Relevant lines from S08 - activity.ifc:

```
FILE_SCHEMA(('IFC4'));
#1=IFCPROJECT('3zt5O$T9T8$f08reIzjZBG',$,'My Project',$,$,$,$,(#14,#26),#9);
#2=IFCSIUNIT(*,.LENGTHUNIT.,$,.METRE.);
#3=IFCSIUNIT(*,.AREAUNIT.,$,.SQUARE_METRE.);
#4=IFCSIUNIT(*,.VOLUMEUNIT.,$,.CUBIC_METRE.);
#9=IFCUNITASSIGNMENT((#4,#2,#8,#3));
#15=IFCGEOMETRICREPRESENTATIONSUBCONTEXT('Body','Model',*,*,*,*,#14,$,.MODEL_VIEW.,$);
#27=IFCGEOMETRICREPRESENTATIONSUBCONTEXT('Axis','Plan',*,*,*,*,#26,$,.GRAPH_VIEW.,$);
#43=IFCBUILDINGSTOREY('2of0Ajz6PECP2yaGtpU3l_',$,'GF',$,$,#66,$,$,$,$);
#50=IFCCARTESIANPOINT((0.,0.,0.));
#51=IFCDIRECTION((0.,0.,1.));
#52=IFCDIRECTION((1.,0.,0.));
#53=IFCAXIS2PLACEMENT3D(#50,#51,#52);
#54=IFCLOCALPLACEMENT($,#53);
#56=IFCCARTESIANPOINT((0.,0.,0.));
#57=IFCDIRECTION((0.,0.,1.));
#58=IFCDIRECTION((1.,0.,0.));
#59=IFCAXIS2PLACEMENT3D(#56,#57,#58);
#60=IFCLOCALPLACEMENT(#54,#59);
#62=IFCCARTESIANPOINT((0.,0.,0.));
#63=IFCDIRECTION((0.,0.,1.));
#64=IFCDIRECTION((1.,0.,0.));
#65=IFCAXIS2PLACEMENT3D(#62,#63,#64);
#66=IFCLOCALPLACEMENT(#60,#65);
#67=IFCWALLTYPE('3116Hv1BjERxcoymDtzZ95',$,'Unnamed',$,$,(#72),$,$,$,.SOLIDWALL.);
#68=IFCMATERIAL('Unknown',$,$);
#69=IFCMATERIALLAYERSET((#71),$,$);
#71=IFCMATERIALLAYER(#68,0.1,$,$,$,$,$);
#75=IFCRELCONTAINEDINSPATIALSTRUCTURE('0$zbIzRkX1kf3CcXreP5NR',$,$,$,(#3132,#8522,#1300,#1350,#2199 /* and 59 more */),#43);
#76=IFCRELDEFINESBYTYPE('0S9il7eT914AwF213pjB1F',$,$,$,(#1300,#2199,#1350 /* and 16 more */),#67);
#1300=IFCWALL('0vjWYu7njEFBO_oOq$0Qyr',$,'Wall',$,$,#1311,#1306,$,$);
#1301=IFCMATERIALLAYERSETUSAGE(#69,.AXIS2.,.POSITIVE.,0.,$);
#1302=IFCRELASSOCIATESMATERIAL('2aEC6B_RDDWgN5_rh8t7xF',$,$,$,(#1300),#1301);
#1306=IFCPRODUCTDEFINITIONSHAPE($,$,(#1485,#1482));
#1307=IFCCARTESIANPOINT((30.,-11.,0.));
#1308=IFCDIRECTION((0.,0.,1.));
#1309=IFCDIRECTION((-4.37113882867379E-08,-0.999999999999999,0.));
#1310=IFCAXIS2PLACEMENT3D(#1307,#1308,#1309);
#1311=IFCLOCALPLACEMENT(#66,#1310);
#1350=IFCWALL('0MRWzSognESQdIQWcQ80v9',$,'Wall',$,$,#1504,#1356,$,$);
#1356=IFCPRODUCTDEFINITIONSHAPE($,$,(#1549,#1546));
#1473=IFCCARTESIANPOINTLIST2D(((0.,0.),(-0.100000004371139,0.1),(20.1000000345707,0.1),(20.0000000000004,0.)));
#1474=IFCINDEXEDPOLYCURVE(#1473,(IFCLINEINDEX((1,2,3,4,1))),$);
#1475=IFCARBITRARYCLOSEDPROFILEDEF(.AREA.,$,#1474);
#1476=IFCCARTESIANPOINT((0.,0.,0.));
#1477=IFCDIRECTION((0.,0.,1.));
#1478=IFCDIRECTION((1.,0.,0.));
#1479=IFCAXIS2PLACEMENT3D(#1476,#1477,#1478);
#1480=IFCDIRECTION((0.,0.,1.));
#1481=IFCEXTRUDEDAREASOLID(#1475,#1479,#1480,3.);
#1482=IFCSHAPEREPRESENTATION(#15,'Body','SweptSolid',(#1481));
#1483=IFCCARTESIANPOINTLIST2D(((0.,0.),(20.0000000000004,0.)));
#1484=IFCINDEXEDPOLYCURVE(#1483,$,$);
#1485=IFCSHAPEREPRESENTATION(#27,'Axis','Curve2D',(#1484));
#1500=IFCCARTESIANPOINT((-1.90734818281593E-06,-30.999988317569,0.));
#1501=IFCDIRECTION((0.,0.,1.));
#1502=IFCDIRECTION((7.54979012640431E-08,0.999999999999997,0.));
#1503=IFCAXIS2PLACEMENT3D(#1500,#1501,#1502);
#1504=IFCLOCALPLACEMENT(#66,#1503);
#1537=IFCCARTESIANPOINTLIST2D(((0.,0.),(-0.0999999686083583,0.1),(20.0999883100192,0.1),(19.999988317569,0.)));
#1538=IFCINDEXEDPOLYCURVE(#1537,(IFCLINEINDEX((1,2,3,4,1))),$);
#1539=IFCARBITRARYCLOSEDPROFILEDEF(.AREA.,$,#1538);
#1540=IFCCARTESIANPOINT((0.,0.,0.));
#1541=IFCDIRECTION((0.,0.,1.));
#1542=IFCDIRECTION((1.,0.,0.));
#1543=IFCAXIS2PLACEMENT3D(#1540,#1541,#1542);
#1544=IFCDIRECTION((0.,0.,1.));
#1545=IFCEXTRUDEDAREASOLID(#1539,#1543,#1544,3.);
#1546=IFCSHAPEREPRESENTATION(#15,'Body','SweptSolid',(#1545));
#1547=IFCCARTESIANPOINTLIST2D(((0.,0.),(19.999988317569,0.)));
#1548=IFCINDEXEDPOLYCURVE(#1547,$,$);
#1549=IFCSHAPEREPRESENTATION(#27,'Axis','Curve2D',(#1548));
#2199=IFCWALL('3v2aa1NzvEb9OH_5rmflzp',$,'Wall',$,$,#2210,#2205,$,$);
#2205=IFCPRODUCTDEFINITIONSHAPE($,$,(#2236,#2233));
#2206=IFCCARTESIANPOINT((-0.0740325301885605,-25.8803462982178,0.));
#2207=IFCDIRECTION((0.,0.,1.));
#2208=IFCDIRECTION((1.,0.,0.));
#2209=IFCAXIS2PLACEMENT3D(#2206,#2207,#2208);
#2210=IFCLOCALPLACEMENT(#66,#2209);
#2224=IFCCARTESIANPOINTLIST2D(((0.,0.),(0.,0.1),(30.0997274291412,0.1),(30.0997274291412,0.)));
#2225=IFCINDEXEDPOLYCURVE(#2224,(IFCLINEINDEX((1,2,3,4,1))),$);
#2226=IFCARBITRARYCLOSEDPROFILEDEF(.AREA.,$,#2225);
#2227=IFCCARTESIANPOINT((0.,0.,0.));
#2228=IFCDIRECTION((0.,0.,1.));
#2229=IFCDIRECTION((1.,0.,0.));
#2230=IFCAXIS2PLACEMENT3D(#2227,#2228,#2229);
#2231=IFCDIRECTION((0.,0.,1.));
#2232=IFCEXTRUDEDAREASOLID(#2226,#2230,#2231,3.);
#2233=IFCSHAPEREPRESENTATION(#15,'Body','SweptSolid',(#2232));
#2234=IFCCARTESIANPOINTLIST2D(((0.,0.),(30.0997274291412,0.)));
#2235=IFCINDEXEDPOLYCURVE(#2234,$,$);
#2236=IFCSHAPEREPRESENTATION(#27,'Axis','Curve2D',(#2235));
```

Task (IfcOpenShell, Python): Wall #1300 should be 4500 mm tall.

```python
import ifcopenshell
import ifcopenshell.geom
import ifcopenshell.util.representation
import ifcopenshell.util.shape

model = ifcopenshell.open("S08 - activity.ifc")
settings = ifcopenshell.geom.settings()


def volume(element):
    """Net volume in cubic metres, openings subtracted."""
    shape = ifcopenshell.geom.create_shape(settings, element)
    return ifcopenshell.util.shape.get_volume(shape.geometry)


wall = model.by_guid("0vjWYu7njEFBO_oOq$0Qyr")
before = volume(wall)

body = ifcopenshell.util.representation.get_representation(wall, "Model", "Body")
solid = body.Items[0]
old_height = solid.Depth
solid.Depth = 4.5
after = volume(wall)

print(f"height {old_height:g} -> {solid.Depth:g}, volume {before:.3f} -> {after:.3f} m3")

model.write("S08 - activity_v2.ifc")
```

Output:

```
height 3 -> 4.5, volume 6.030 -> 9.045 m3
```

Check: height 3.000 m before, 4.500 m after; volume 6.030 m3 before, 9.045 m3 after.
